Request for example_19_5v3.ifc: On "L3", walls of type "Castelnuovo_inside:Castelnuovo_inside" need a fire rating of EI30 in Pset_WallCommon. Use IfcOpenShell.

First a look at what the model holds.

```python
import ifcopenshell
import ifcopenshell.util.element

model = ifcopenshell.open("example_19_5v3.ifc")
print(model.schema)
storey = next(s for s in model.by_type("IfcBuildingStorey") if s.Name == "L3")
walls = [e for e in ifcopenshell.util.element.get_decomposition(storey) if e.is_a("IfcWall")]
seen = {}
for e in walls:
    element_type = ifcopenshell.util.element.get_type(e)
    key = (element_type.Name if element_type != e and element_type else None, ifcopenshell.util.element.get_pset(e, "Pset_WallCommon", "FireRating"))
    seen[key] = seen.get(key, 0) + 1
for (name, value), count in sorted(seen.items(), key=str):
    print(count, "x", name, "|", value)
```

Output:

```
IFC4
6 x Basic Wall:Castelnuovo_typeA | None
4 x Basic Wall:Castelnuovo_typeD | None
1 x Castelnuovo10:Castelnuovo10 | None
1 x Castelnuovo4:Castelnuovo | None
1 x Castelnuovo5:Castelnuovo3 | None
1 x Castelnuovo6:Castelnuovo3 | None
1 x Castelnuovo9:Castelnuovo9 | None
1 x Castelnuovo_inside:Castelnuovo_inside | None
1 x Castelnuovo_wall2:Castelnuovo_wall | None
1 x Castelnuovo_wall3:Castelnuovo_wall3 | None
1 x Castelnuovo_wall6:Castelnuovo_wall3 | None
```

```python
import ifcopenshell
import ifcopenshell.api.pset
import ifcopenshell.util.element

model = ifcopenshell.open("example_19_5v3.ifc")

storey = next(s for s in model.by_type("IfcBuildingStorey") if s.Name == "L3")
walls = [e for e in ifcopenshell.util.element.get_decomposition(storey) if e.is_a("IfcWall")]

count = 0
for e in walls:
    element_type = ifcopenshell.util.element.get_type(e)
    if element_type in (None, e) or element_type.Name != "Castelnuovo_inside:Castelnuovo_inside":
        continue
    # add_pset returns the element's existing set when there is one.
    pset = ifcopenshell.api.pset.add_pset(model, product=e, name="Pset_WallCommon")
    ifcopenshell.api.pset.edit_pset(model, pset=pset, properties={"FireRating": "EI30"})
    count += 1

print(count, "walls updated")

model.write("example_19_5v3_v2.ifc")
```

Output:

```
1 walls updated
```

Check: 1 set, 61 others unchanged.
